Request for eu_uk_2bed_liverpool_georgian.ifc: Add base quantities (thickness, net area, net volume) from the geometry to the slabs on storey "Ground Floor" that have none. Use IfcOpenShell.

First a look at what the model holds.

```python
import ifcopenshell
import ifcopenshell.util.element
import ifcopenshell.util.unit

model = ifcopenshell.open("eu_uk_2bed_liverpool_georgian.ifc")
print(model.schema)
for unit_type in ("LENGTHUNIT", "AREAUNIT", "VOLUMEUNIT"):
    print(unit_type, ifcopenshell.util.unit.calculate_unit_scale(model, unit_type))
storey = next(s for s in model.by_type("IfcBuildingStorey") if s.Name == "Ground Floor")
slabs = [e for e in ifcopenshell.util.element.get_decomposition(storey) if e.is_a("IfcSlab")]
for e in sorted(slabs, key=lambda e: e.id()):
    print(e.id(), e.is_a(), e.Name, list(ifcopenshell.util.element.get_psets(e, qtos_only=True)), sep=" | ")
```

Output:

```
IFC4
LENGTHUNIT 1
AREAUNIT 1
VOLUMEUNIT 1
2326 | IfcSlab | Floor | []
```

```python
import ifcopenshell
import ifcopenshell.api.pset
import ifcopenshell.geom
import ifcopenshell.util.element
import ifcopenshell.util.shape
import ifcopenshell.util.unit

model = ifcopenshell.open("eu_uk_2bed_liverpool_georgian.ifc")
unit_scale = ifcopenshell.util.unit.calculate_unit_scale(model)
area_scale = ifcopenshell.util.unit.calculate_unit_scale(model, "AREAUNIT")
volume_scale = ifcopenshell.util.unit.calculate_unit_scale(model, "VOLUMEUNIT")
settings = ifcopenshell.geom.settings()

storey = next(s for s in model.by_type("IfcBuildingStorey") if s.Name == "Ground Floor")
slabs = [e for e in ifcopenshell.util.element.get_decomposition(storey) if e.is_a("IfcSlab")]

for e in sorted(slabs, key=lambda e: e.id()):
    if ifcopenshell.util.element.get_psets(e, qtos_only=True, should_inherit=False):
        continue
    # Geometry comes back in metres, in the element's own axes.
    shape = ifcopenshell.geom.create_shape(settings, e)
    values = {
        "Width": ifcopenshell.util.shape.get_z(shape.geometry) / unit_scale,
        "NetArea": ifcopenshell.util.shape.get_footprint_area(shape.geometry) / area_scale,
        "NetVolume": ifcopenshell.util.shape.get_volume(shape.geometry) / volume_scale,
    }
    qto = ifcopenshell.api.pset.add_qto(model, product=e, name="Qto_SlabBaseQuantities")
    ifcopenshell.api.pset.edit_qto(model, qto=qto, properties=values)
    print(e.id(), {k: round(v, 3) for k, v in values.items()})

model.write("eu_uk_2bed_liverpool_georgian_v2.ifc")
```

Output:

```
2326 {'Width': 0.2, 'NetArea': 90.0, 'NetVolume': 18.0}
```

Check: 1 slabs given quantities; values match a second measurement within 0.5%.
